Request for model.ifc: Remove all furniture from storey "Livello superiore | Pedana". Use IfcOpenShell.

First a look at what the model holds.

```python
import ifcopenshell
import ifcopenshell.util.element

model = ifcopenshell.open("model.ifc")
print(model.schema)
storey = next(s for s in model.by_type("IfcBuildingStorey") if s.Name == "Livello superiore | Pedana")
furniture = [e for e in ifcopenshell.util.element.get_decomposition(storey) if e.is_a("IfcFurnishingElement")]
seen = {}
for e in furniture:
    element_type = ifcopenshell.util.element.get_type(e)
    name = element_type.Name if element_type not in (None, e) else None
    seen[name] = seen.get(name, 0) + 1
for name, count in sorted(seen.items(), key=str):
    print(count, "x", name)
```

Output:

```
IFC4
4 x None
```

```python
import ifcopenshell
import ifcopenshell.api.root
import ifcopenshell.util.element

model = ifcopenshell.open("model.ifc")

storey = next(s for s in model.by_type("IfcBuildingStorey") if s.Name == "Livello superiore | Pedana")
furniture = [e for e in ifcopenshell.util.element.get_decomposition(storey) if e.is_a("IfcFurnishingElement")]

for e in furniture:
    ifcopenshell.api.root.remove_product(model, product=e)
print(len(furniture), "removed")

model.write("model-out.ifc")
```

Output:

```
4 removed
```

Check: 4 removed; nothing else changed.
